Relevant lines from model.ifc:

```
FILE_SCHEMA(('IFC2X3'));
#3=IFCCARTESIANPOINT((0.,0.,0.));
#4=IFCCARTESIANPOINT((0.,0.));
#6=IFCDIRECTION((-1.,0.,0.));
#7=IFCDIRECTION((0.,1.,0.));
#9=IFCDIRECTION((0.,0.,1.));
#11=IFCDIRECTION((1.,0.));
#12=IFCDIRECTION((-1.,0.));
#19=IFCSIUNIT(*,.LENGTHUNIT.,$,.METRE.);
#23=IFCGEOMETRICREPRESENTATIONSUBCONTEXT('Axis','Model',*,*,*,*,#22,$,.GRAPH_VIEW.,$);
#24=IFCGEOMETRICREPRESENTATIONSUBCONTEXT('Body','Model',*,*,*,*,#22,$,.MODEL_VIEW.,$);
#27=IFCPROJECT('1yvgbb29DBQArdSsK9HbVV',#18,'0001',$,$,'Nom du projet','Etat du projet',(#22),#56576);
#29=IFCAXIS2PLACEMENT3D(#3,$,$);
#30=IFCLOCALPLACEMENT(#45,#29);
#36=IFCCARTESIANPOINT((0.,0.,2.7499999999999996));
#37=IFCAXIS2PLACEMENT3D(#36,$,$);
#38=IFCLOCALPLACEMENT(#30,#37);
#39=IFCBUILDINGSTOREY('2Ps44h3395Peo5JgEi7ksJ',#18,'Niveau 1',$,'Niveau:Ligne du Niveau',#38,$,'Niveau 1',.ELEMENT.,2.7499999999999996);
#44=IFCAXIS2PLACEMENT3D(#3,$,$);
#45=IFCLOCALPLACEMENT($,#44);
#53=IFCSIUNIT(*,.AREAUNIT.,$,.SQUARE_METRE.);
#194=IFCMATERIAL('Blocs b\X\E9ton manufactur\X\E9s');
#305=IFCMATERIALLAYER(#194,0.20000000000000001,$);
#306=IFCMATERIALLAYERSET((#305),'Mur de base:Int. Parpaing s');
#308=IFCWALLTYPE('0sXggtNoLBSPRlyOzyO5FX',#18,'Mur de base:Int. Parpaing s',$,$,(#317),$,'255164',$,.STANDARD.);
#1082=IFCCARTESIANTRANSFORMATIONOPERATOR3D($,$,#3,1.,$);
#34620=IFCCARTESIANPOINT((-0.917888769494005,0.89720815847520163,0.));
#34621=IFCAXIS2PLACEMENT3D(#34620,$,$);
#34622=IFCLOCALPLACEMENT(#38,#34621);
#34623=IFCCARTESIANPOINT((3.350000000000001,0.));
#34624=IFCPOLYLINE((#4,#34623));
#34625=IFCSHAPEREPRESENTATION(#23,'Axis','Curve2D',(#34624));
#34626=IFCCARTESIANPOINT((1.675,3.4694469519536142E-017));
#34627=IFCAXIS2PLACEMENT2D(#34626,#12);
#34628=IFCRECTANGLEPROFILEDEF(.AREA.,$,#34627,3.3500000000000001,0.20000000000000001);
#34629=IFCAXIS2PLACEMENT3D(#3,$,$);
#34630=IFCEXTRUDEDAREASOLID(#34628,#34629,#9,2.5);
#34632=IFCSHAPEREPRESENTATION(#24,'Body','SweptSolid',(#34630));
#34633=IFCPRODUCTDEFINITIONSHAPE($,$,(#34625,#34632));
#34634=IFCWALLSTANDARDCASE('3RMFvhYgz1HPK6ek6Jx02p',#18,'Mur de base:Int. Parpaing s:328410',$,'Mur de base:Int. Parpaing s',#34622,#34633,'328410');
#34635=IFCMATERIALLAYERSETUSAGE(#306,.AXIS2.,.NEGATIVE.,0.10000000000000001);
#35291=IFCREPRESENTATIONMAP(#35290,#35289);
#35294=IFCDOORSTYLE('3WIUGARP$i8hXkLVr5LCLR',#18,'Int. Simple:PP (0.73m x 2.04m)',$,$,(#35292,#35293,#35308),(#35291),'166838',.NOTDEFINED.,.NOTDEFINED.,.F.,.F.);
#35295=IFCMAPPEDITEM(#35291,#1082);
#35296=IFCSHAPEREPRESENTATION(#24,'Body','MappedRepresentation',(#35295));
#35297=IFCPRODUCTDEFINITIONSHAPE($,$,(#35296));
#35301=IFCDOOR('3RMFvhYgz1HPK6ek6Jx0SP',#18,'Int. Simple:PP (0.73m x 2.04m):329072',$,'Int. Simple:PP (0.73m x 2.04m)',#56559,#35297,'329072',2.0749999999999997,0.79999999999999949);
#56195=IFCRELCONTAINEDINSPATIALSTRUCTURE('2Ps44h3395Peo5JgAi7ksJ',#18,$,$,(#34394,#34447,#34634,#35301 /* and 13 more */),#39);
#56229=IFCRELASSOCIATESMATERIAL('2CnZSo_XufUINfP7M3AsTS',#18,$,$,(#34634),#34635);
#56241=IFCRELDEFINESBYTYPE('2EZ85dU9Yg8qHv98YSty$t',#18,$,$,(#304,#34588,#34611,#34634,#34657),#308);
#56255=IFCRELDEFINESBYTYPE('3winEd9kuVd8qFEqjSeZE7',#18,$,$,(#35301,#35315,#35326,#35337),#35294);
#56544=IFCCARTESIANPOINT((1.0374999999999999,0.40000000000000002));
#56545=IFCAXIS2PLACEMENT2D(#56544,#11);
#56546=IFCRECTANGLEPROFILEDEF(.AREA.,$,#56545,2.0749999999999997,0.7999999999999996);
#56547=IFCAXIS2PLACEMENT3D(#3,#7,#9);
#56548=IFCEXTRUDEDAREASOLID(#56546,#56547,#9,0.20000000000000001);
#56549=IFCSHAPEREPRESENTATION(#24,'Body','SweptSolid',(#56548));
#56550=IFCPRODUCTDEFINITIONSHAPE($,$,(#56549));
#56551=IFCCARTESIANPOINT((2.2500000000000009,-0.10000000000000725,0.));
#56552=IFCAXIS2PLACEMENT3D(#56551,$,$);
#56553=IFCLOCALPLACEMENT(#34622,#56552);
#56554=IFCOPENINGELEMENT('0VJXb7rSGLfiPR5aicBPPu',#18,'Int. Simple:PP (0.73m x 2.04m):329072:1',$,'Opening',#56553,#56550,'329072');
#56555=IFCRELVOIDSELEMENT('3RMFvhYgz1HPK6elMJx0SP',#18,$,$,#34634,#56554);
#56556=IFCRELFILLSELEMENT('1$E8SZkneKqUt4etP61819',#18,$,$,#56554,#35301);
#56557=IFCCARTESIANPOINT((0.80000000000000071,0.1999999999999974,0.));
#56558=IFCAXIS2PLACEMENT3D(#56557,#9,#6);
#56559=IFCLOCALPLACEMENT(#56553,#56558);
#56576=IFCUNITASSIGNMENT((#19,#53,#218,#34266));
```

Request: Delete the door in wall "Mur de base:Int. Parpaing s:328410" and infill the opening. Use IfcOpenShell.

```python
import ifcopenshell
import ifcopenshell.api.feature
import ifcopenshell.api.root
import ifcopenshell.geom
import ifcopenshell.util.shape

model = ifcopenshell.open("model.ifc")
settings = ifcopenshell.geom.settings()


def volume(element):
    """Net volume in cubic metres, openings subtracted."""
    shape = ifcopenshell.geom.create_shape(settings, element)
    return ifcopenshell.util.shape.get_volume(shape.geometry)


door = model.by_guid("3RMFvhYgz1HPK6ek6Jx0SP")
opening = door.FillsVoids[0].RelatingOpeningElement
wall = opening.VoidsElements[0].RelatingBuildingElement
before = volume(wall)

ifcopenshell.api.root.remove_product(model, product=door)
ifcopenshell.api.feature.remove_feature(model, feature=opening)

after = volume(wall)

print(f"wall volume {before:.3f} -> {after:.3f} m3")

model.write("model_v2.ifc")
```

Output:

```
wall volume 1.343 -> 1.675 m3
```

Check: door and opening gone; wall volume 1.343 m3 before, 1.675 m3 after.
